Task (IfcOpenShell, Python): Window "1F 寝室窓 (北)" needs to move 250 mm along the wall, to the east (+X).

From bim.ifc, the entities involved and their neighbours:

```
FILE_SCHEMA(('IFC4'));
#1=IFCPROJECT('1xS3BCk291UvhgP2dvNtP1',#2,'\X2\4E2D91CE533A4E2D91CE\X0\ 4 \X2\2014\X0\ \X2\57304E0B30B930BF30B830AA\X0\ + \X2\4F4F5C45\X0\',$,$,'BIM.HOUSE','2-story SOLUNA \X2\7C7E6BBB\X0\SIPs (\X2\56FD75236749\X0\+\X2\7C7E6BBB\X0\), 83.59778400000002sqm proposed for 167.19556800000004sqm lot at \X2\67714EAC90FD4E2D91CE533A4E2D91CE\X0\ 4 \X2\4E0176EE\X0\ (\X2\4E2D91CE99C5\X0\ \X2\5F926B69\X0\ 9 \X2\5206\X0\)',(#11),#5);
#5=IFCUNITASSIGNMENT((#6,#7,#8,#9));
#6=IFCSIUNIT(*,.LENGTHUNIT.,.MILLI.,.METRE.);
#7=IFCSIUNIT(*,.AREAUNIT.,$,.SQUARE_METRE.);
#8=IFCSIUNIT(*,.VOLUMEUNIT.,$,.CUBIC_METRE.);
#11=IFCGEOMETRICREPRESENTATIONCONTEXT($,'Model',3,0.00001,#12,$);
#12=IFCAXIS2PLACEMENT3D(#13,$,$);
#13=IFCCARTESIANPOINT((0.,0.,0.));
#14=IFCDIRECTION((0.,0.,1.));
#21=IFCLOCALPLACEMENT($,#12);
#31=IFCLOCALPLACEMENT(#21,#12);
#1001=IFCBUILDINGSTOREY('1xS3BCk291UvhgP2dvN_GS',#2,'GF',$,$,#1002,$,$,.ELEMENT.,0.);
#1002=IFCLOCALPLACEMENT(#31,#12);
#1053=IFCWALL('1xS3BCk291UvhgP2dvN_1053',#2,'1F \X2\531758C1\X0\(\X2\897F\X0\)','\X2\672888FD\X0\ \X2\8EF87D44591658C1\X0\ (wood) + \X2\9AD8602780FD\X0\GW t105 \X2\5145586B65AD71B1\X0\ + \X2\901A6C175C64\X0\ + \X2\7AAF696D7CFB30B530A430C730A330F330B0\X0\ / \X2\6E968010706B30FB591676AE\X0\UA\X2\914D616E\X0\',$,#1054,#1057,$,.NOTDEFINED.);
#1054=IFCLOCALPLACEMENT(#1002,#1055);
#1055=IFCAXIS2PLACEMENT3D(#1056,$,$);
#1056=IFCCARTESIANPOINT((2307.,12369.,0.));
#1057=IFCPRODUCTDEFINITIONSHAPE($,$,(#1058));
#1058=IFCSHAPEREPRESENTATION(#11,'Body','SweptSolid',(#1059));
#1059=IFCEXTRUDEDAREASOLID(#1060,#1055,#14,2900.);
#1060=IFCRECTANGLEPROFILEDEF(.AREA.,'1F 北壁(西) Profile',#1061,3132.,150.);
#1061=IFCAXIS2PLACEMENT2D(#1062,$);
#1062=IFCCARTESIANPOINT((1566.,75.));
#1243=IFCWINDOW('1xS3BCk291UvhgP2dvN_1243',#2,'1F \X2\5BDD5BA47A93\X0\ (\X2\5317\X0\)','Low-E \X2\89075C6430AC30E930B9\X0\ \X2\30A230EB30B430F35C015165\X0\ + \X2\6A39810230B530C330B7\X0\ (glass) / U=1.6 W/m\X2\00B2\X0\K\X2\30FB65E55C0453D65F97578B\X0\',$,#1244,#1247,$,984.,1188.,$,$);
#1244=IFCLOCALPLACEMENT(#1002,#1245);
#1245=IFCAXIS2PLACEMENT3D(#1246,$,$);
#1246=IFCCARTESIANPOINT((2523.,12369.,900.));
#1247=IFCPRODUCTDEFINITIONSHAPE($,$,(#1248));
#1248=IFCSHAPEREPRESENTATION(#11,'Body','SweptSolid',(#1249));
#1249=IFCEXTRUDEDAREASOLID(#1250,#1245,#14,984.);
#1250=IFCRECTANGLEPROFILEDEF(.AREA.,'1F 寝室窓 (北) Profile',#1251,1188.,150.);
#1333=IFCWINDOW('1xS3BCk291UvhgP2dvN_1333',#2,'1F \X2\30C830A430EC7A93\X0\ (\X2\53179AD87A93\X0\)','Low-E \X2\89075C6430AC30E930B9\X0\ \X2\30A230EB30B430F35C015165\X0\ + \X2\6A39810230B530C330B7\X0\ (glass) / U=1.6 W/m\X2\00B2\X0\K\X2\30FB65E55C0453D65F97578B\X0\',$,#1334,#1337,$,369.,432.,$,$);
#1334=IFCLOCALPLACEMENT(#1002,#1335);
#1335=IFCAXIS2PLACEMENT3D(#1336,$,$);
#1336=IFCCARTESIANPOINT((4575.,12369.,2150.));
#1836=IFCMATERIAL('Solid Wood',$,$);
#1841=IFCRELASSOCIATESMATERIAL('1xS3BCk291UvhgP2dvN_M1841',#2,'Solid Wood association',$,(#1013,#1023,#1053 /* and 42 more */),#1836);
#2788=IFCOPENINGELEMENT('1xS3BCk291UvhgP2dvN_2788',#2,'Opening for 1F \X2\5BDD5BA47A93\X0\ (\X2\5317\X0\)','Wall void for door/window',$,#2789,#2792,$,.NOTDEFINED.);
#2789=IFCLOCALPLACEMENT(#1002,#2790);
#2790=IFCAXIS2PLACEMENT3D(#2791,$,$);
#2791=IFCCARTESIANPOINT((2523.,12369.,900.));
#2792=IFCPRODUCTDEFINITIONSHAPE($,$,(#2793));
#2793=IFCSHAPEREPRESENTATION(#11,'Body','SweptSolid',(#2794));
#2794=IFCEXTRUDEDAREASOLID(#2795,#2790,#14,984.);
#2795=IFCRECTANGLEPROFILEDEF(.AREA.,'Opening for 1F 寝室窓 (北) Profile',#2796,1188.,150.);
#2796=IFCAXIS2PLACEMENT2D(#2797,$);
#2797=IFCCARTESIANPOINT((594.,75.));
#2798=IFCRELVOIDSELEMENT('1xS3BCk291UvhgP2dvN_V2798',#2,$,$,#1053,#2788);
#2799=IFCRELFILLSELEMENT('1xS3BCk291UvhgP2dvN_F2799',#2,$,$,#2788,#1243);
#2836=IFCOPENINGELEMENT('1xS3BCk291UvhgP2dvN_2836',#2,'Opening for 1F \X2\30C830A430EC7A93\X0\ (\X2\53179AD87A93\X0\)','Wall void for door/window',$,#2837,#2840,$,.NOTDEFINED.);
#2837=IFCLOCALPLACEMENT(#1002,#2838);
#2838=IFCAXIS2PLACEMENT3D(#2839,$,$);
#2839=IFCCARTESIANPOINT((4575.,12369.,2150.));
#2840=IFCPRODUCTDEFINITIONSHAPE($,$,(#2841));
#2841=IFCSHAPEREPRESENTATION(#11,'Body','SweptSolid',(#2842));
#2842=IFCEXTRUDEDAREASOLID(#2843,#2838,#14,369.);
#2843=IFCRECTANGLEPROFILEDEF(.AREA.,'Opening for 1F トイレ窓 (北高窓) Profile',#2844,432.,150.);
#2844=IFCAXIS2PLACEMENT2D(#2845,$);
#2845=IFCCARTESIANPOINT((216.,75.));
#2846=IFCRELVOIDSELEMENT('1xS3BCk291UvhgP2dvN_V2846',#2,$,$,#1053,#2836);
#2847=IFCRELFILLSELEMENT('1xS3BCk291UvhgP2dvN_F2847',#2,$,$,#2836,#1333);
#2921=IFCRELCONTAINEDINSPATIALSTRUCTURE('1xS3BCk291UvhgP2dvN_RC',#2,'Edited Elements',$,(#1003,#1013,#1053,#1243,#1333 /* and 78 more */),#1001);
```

```python
import ifcopenshell
import ifcopenshell.api.geometry
import ifcopenshell.util.placement
import ifcopenshell.util.unit

model = ifcopenshell.open("bim.ifc")
unit_scale = ifcopenshell.util.unit.calculate_unit_scale(model)

window = model.by_guid("1xS3BCk291UvhgP2dvN_1243")
opening = window.FillsVoids[0].RelatingOpeningElement
wall = opening.VoidsElements[0].RelatingBuildingElement

wall_matrix = ifcopenshell.util.placement.get_local_placement(wall.ObjectPlacement)
shift = wall_matrix[:3, 0] * 0.25 / unit_scale
before = ifcopenshell.util.placement.get_local_placement(window.ObjectPlacement)[:3, 3].copy()

# The window is not placed relative to its opening, so move both.
for product in (opening, window):
    matrix = ifcopenshell.util.placement.get_local_placement(product.ObjectPlacement)
    matrix[:3, 3] += shift
    ifcopenshell.api.geometry.edit_object_placement(model, product=product, matrix=matrix, is_si=False)

after = ifcopenshell.util.placement.get_local_placement(window.ObjectPlacement)[:3, 3]
print("window moved by", (after - before).round(3) + 0.0)

model.write("bim_v2.ifc")
```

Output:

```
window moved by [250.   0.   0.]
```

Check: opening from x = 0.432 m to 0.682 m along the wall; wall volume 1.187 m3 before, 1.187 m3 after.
